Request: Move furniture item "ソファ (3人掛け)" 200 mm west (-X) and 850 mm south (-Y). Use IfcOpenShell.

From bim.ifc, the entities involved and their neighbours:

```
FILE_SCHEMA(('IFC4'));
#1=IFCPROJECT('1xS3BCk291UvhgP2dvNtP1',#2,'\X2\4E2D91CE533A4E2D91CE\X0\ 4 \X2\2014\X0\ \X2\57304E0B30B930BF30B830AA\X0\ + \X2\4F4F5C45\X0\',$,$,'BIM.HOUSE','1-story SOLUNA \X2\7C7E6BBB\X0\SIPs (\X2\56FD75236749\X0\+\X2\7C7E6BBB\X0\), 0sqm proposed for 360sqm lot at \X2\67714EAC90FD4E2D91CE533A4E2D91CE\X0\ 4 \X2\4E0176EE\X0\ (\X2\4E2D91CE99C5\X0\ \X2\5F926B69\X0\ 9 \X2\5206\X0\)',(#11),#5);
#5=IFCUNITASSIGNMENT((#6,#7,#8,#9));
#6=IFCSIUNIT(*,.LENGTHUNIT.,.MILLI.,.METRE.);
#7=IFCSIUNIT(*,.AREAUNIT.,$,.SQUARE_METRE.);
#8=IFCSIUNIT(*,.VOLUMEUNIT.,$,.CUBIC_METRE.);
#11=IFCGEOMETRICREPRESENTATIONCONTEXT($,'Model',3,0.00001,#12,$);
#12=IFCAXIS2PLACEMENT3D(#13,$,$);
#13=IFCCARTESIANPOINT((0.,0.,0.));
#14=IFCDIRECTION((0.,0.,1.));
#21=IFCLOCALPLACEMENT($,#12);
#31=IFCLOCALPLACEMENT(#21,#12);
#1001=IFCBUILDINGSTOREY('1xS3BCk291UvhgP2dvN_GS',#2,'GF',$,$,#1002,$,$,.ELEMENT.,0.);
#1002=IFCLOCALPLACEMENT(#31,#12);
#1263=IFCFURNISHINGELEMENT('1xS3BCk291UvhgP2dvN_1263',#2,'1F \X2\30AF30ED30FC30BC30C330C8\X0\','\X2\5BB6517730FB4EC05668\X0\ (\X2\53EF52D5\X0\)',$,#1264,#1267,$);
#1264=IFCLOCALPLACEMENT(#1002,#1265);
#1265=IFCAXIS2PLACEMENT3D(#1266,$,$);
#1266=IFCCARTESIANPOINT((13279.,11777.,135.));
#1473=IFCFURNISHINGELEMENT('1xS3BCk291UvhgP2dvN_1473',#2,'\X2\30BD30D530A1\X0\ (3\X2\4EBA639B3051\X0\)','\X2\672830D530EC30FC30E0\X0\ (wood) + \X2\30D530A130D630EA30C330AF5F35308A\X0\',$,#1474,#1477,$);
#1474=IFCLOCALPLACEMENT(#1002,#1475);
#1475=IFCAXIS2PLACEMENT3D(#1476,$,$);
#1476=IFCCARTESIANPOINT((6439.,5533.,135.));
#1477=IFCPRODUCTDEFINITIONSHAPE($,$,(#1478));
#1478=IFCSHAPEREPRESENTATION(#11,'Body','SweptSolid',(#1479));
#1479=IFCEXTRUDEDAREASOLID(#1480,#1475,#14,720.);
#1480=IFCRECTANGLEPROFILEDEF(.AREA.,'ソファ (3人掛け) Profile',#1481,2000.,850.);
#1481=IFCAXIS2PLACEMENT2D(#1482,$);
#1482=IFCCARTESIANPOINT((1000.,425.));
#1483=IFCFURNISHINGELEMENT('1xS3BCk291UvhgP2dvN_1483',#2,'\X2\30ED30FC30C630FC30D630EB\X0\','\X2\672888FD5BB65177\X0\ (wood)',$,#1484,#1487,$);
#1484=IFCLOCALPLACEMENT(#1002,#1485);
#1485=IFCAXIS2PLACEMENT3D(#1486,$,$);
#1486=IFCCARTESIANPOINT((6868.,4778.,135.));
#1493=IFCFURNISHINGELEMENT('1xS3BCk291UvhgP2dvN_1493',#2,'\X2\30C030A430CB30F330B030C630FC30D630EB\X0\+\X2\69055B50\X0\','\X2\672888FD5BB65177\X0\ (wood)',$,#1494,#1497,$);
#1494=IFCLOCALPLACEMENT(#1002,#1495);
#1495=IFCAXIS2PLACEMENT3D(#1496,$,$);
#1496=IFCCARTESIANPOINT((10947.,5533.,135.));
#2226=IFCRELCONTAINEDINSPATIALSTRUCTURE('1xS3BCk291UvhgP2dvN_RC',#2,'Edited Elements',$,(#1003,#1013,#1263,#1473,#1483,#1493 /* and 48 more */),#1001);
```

```python
import ifcopenshell
import ifcopenshell.api.geometry
import ifcopenshell.util.placement

model = ifcopenshell.open("bim.ifc")

item = model.by_guid("1xS3BCk291UvhgP2dvN_1473")
matrix = ifcopenshell.util.placement.get_local_placement(item.ObjectPlacement)
matrix[0, 3] -= 200.0
matrix[1, 3] -= 850.0
ifcopenshell.api.geometry.edit_object_placement(model, product=item, matrix=matrix, is_si=False)

print(ifcopenshell.util.placement.get_local_placement(item.ObjectPlacement).round(3) + 0.0)

model.write("bim-out.ifc")
```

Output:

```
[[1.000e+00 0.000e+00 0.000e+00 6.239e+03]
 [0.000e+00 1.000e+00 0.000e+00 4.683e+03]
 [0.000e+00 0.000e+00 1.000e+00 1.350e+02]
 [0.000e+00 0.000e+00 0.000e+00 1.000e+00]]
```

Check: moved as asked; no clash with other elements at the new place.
